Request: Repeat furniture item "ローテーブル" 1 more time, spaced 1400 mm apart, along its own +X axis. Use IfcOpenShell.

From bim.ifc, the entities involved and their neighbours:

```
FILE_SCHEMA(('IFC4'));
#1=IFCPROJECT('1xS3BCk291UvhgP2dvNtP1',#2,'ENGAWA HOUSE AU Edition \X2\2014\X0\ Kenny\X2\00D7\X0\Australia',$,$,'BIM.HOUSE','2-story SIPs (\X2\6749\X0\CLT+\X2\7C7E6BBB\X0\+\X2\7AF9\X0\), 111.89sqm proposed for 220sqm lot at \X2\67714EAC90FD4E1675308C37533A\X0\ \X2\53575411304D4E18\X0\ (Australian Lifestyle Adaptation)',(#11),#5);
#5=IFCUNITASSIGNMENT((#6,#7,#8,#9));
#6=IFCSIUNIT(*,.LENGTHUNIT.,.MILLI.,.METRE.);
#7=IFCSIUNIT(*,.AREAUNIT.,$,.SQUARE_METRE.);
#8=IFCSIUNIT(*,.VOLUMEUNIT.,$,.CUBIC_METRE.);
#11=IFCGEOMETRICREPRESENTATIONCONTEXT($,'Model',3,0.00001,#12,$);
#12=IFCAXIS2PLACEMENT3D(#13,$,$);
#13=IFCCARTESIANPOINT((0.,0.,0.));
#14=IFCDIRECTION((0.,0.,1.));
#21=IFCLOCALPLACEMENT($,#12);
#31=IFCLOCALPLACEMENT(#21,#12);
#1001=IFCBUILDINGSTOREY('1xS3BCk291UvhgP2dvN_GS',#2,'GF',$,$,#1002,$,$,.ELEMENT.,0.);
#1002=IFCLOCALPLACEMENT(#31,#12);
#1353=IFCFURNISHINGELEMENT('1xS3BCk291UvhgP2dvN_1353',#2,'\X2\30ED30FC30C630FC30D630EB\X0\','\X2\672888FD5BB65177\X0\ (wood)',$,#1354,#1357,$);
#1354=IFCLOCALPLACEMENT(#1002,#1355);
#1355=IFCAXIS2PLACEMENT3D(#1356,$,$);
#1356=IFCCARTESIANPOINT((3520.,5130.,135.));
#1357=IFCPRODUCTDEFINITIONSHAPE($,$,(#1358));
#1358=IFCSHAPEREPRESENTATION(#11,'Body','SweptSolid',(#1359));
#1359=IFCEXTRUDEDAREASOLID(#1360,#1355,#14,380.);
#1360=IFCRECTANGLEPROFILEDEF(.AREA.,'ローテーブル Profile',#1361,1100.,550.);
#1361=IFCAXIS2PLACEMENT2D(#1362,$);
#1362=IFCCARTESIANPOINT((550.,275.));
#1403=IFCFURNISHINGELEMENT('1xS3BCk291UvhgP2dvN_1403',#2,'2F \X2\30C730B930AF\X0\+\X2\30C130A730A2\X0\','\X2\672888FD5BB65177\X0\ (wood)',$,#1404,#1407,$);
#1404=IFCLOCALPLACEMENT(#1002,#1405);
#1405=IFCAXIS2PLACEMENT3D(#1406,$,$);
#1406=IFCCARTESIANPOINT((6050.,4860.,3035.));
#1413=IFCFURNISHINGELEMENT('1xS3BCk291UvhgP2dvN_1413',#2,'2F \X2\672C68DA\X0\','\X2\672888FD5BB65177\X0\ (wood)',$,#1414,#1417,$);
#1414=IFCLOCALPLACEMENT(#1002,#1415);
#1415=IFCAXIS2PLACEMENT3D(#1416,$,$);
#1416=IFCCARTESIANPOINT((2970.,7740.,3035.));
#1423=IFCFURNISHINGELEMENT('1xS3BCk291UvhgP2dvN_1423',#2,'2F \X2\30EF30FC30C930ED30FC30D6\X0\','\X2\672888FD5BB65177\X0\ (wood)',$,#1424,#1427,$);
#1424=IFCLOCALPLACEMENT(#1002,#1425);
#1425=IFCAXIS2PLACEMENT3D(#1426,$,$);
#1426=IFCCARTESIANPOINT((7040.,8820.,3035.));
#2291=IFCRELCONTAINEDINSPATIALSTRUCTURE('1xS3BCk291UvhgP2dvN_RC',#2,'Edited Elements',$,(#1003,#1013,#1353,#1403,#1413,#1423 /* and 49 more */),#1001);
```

```python
import ifcopenshell
import ifcopenshell.api.geometry
import ifcopenshell.api.root
import ifcopenshell.util.element
import ifcopenshell.util.placement
import ifcopenshell.util.unit

model = ifcopenshell.open("bim.ifc")
unit_scale = ifcopenshell.util.unit.calculate_unit_scale(model)


def reuse_history(source, copy):
    """copy_class also copies each property set's owner history, people and application; keep the originals."""
    for rel in copy.IsDefinedBy:
        if rel.is_a("IfcRelDefinesByProperties") and (history := rel.RelatingPropertyDefinition.OwnerHistory):
            rel.RelatingPropertyDefinition.OwnerHistory = source.OwnerHistory
            ifcopenshell.util.element.remove_deep2(model, history)


source = model.by_id(1353)
base = ifcopenshell.util.placement.get_local_placement(source.ObjectPlacement)
step = base[:3, 0] * 1.4 / unit_scale

for i in range(1, 2):
    copy = ifcopenshell.api.root.copy_class(model, product=source)
    copy.Representation = ifcopenshell.util.element.copy_deep(
        model, source.Representation, exclude=["IfcGeometricRepresentationContext", "IfcRepresentationMap"]
    )
    reuse_history(source, copy)
    matrix = base.copy()
    matrix[:3, 3] += i * step
    print("added at", matrix[:3, 3].round(3) + 0.0)
    ifcopenshell.api.geometry.edit_object_placement(model, product=copy, matrix=matrix, is_si=False)

model.write("bim_rev.ifc")
```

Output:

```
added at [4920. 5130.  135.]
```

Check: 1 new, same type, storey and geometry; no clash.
